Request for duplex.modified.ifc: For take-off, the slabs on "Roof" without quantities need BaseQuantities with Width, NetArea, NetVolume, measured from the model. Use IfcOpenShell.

First a look at what the model holds.

```python
import ifcopenshell
import ifcopenshell.util.element
import ifcopenshell.util.unit

model = ifcopenshell.open("duplex.modified.ifc")
print(model.schema)
for unit_type in ("LENGTHUNIT", "AREAUNIT", "VOLUMEUNIT"):
    print(unit_type, ifcopenshell.util.unit.calculate_unit_scale(model, unit_type))
storey = next(s for s in model.by_type("IfcBuildingStorey") if s.Name == "Roof")
slabs = [e for e in ifcopenshell.util.element.get_decomposition(storey) if e.is_a("IfcSlab")]
for e in sorted(slabs, key=lambda e: e.id()):
    print(e.id(), e.is_a(), e.Name, list(ifcopenshell.util.element.get_psets(e, qtos_only=True)), sep=" | ")
```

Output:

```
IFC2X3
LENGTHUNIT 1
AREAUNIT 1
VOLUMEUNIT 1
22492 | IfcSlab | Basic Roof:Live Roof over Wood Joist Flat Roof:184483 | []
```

```python
import ifcopenshell
import ifcopenshell.api.pset
import ifcopenshell.geom
import ifcopenshell.util.element
import ifcopenshell.util.shape
import ifcopenshell.util.unit

model = ifcopenshell.open("duplex.modified.ifc")
unit_scale = ifcopenshell.util.unit.calculate_unit_scale(model)
area_scale = ifcopenshell.util.unit.calculate_unit_scale(model, "AREAUNIT")
volume_scale = ifcopenshell.util.unit.calculate_unit_scale(model, "VOLUMEUNIT")
settings = ifcopenshell.geom.settings()

storey = next(s for s in model.by_type("IfcBuildingStorey") if s.Name == "Roof")
slabs = [e for e in ifcopenshell.util.element.get_decomposition(storey) if e.is_a("IfcSlab")]

for e in sorted(slabs, key=lambda e: e.id()):
    if ifcopenshell.util.element.get_psets(e, qtos_only=True, should_inherit=False):
        continue
    # Geometry comes back in metres, in the element's own axes.
    shape = ifcopenshell.geom.create_shape(settings, e)
    values = {
        "Width": ifcopenshell.util.shape.get_z(shape.geometry) / unit_scale,
        "NetArea": ifcopenshell.util.shape.get_footprint_area(shape.geometry) / area_scale,
        "NetVolume": ifcopenshell.util.shape.get_volume(shape.geometry) / volume_scale,
    }
    qto = ifcopenshell.api.pset.add_qto(model, product=e, name="BaseQuantities")
    ifcopenshell.api.pset.edit_qto(model, qto=qto, properties=values)
    print(e.id(), {k: round(v, 3) for k, v in values.items()})

model.write("duplex.modified_edited.ifc")
```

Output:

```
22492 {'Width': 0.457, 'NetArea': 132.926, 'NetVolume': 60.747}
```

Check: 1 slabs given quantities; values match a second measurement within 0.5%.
